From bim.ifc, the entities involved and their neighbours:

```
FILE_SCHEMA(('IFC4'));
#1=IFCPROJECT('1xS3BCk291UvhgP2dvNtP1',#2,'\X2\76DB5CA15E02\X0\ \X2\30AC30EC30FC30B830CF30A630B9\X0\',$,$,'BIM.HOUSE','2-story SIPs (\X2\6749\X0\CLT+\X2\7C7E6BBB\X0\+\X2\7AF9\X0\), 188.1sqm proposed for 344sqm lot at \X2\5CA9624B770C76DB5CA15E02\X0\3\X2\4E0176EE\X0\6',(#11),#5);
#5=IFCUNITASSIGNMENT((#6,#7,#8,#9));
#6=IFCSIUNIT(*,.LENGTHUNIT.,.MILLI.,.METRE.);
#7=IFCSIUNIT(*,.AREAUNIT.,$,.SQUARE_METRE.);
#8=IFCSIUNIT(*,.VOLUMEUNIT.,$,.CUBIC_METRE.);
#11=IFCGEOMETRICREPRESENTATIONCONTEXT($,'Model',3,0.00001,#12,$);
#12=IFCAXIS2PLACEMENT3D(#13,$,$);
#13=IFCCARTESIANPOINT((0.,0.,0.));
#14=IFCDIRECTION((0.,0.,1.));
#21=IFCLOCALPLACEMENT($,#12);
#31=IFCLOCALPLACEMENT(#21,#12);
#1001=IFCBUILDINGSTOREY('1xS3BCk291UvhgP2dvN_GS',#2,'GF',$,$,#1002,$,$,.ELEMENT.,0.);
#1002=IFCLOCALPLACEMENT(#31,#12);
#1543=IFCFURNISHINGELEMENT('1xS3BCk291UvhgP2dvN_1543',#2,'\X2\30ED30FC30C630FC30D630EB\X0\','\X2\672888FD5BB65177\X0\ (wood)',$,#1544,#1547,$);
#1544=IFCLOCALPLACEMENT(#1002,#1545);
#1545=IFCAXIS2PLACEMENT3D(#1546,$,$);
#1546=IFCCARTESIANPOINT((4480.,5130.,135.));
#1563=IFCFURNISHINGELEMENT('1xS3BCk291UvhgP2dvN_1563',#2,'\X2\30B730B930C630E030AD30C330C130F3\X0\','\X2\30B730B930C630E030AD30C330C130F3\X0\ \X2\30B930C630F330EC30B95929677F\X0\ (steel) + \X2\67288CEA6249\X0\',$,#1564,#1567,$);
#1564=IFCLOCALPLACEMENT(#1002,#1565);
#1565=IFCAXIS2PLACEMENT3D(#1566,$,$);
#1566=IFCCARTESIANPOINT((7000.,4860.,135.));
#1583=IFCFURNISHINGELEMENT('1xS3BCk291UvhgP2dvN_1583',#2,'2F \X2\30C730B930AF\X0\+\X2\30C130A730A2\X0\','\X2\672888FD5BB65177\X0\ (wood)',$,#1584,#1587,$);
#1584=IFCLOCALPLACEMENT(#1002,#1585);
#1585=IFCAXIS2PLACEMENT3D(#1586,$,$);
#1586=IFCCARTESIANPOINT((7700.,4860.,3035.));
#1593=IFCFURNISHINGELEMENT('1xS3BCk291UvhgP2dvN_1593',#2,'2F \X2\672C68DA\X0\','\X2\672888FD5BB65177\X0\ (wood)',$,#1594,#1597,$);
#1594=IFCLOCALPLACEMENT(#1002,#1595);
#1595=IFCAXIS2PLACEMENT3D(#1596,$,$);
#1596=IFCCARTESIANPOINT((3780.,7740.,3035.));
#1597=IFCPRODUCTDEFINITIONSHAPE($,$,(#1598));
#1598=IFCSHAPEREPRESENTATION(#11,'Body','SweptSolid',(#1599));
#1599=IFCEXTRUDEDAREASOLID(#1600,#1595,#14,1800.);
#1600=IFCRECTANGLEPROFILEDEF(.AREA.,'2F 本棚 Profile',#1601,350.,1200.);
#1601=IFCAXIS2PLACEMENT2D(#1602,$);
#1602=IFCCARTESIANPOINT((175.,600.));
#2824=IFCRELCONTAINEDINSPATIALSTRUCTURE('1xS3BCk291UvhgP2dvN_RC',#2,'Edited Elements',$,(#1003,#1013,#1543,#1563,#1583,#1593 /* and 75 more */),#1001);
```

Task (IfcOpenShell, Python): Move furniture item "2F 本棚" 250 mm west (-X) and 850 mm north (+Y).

```python
import ifcopenshell
import ifcopenshell.api.geometry
import ifcopenshell.util.placement
import ifcopenshell.util.unit

model = ifcopenshell.open("bim.ifc")
unit_scale = ifcopenshell.util.unit.calculate_unit_scale(model)

item = model.by_id(1593)
matrix = ifcopenshell.util.placement.get_local_placement(item.ObjectPlacement)
matrix[0, 3] -= 0.25 / unit_scale
matrix[1, 3] += 0.85 / unit_scale
ifcopenshell.api.geometry.edit_object_placement(model, product=item, matrix=matrix, is_si=False)

print(ifcopenshell.util.placement.get_local_placement(item.ObjectPlacement).round(3) + 0.0)

model.write("bim-out.ifc")
```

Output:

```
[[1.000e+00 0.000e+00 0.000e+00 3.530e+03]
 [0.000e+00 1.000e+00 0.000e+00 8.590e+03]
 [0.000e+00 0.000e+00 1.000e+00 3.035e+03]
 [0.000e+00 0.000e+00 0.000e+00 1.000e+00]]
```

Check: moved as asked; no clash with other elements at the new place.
